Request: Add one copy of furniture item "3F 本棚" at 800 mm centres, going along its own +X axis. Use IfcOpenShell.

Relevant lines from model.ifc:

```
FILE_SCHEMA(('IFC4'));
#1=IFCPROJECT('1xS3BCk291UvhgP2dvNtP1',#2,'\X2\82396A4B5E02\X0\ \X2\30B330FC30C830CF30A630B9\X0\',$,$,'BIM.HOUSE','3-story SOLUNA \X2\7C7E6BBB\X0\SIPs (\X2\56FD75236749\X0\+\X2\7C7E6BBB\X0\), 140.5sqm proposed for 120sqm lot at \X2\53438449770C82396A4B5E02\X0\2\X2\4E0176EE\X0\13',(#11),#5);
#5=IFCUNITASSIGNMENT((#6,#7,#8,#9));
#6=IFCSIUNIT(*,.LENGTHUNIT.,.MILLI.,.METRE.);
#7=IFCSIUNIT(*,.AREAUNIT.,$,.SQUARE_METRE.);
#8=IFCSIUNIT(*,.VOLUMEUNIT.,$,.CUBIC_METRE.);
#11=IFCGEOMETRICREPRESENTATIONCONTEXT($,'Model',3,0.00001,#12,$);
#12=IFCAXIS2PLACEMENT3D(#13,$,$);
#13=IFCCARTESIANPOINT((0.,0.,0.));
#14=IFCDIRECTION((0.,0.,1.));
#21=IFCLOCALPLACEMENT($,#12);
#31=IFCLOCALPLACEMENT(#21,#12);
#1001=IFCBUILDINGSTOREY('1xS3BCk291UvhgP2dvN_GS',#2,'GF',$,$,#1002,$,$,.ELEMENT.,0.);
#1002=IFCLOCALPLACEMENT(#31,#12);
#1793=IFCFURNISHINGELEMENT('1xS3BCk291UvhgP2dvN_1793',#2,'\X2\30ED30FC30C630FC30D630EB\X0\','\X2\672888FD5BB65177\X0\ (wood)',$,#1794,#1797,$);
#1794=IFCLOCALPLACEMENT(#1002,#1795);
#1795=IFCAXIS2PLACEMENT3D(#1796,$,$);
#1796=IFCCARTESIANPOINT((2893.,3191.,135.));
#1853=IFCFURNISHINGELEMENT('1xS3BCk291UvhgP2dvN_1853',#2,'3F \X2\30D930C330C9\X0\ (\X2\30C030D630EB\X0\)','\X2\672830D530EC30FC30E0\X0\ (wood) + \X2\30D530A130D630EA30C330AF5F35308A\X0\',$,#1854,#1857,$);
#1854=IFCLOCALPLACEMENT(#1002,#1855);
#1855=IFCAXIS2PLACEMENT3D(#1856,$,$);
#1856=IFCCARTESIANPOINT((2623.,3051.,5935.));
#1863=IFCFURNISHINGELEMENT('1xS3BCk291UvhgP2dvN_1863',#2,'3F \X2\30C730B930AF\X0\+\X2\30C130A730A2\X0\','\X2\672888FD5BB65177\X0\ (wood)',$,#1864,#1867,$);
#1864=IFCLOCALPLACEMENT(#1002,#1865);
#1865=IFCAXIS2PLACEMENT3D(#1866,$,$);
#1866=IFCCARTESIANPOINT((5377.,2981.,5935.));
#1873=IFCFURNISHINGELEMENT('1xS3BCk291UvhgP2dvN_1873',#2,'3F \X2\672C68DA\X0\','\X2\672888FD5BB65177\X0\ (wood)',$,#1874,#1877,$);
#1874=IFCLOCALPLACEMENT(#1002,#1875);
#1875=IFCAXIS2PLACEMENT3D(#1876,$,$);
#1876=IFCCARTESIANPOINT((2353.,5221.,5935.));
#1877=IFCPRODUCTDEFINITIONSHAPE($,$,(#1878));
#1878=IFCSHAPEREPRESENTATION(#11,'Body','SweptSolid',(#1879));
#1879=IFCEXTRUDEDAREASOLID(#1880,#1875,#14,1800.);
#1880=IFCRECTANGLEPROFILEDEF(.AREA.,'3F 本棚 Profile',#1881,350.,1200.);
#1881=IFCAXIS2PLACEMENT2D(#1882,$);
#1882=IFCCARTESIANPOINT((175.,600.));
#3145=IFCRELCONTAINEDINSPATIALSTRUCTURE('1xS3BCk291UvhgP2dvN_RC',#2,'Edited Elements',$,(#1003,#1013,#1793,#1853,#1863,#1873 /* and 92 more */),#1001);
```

```python
import ifcopenshell
import ifcopenshell.api.geometry
import ifcopenshell.api.root
import ifcopenshell.util.element
import ifcopenshell.util.placement

model = ifcopenshell.open("model.ifc")


def reuse_history(source, copy):
    """copy_class also copies each property set's owner history, people and application; keep the originals."""
    for rel in copy.IsDefinedBy:
        if rel.is_a("IfcRelDefinesByProperties") and (history := rel.RelatingPropertyDefinition.OwnerHistory):
            rel.RelatingPropertyDefinition.OwnerHistory = source.OwnerHistory
            ifcopenshell.util.element.remove_deep2(model, history)


source = model.by_guid("1xS3BCk291UvhgP2dvN_1873")
base = ifcopenshell.util.placement.get_local_placement(source.ObjectPlacement)
step = base[:3, 0] * 800.0

for i in range(1, 2):
    copy = ifcopenshell.api.root.copy_class(model, product=source)
    copy.Representation = ifcopenshell.util.element.copy_deep(
        model, source.Representation, exclude=["IfcGeometricRepresentationContext", "IfcRepresentationMap"]
    )
    reuse_history(source, copy)
    matrix = base.copy()
    matrix[:3, 3] += i * step
    print("added at", matrix[:3, 3].round(3) + 0.0)
    ifcopenshell.api.geometry.edit_object_placement(model, product=copy, matrix=matrix, is_si=False)

model.write("model_v2.ifc")
```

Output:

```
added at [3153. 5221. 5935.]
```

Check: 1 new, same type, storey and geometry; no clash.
